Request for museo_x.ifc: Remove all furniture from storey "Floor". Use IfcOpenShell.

First a look at what the model holds.

```python
import ifcopenshell
import ifcopenshell.util.element

model = ifcopenshell.open("museo_x.ifc")
print(model.schema)
storey = next(s for s in model.by_type("IfcBuildingStorey") if s.Name == "Floor")
furniture = [e for e in ifcopenshell.util.element.get_decomposition(storey) if e.is_a("IfcFurnishingElement")]
seen = {}
for e in furniture:
    element_type = ifcopenshell.util.element.get_type(e)
    name = element_type.Name if element_type not in (None, e) else None
    seen[name] = seen.get(name, 0) + 1
for name, count in sorted(seen.items(), key=str):
    print(count, "x", name)
```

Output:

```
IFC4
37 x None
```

```python
import ifcopenshell
import ifcopenshell.api.root
import ifcopenshell.util.element

model = ifcopenshell.open("museo_x.ifc")

storey = next(s for s in model.by_type("IfcBuildingStorey") if s.Name == "Floor")
furniture = [e for e in ifcopenshell.util.element.get_decomposition(storey) if e.is_a("IfcFurnishingElement")]

for e in furniture:
    ifcopenshell.api.root.remove_product(model, product=e)
print(len(furniture), "removed")

model.write("museo_x_rev.ifc")
```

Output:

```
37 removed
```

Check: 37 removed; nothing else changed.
